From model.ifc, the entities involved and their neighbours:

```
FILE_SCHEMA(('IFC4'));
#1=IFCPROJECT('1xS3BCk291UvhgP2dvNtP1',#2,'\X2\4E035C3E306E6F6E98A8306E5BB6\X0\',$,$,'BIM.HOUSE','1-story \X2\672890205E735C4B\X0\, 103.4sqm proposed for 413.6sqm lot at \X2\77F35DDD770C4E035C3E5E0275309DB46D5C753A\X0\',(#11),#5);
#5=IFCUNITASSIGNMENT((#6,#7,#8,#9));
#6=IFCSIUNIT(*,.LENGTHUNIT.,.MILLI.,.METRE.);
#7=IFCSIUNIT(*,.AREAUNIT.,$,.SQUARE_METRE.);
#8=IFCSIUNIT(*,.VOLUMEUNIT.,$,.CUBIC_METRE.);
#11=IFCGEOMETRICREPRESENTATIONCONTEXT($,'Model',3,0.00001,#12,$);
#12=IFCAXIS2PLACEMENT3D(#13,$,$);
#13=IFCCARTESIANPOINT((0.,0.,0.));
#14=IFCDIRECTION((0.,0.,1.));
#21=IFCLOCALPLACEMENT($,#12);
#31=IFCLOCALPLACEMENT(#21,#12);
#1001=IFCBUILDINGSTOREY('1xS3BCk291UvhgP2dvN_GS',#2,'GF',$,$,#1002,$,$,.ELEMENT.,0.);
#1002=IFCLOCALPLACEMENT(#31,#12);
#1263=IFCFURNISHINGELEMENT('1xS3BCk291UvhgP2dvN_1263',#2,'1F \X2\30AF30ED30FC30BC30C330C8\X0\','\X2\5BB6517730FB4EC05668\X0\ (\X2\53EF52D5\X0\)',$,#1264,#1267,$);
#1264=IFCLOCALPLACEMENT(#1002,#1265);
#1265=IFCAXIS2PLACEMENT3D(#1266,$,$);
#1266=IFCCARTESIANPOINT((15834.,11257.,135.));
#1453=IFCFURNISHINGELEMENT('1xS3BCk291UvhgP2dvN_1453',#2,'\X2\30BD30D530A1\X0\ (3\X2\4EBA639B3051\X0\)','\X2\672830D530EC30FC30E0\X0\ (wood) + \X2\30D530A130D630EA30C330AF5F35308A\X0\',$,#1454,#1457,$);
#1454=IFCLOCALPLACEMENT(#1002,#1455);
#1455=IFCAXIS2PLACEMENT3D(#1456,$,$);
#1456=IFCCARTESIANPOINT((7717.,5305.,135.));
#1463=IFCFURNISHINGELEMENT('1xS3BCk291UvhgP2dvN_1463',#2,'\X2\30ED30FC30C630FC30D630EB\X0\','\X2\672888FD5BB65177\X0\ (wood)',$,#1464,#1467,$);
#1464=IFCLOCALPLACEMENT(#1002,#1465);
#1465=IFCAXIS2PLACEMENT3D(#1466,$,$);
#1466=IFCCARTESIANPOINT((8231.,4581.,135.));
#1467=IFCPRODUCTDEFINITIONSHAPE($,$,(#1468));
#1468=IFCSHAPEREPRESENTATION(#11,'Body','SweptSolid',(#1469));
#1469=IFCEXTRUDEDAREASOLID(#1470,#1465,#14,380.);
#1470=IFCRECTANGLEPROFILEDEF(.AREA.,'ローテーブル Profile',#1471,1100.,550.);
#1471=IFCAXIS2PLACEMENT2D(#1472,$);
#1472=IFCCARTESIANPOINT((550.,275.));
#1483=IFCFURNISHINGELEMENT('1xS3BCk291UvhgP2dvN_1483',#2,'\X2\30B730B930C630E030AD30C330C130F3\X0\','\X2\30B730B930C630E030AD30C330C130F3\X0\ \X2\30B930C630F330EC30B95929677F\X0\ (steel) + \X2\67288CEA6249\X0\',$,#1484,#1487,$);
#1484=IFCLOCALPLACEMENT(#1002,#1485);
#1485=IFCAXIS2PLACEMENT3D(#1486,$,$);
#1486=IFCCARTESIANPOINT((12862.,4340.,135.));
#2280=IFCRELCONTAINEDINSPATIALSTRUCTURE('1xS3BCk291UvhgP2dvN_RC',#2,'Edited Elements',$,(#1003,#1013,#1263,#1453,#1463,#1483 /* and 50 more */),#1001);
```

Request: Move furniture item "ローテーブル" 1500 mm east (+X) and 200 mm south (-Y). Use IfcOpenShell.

```python
import ifcopenshell
import ifcopenshell.api.geometry
import ifcopenshell.util.placement
import ifcopenshell.util.unit

model = ifcopenshell.open("model.ifc")
unit_scale = ifcopenshell.util.unit.calculate_unit_scale(model)

item = model.by_guid("1xS3BCk291UvhgP2dvN_1463")
matrix = ifcopenshell.util.placement.get_local_placement(item.ObjectPlacement)
matrix[0, 3] += 1.5 / unit_scale
matrix[1, 3] -= 0.2 / unit_scale
ifcopenshell.api.geometry.edit_object_placement(model, product=item, matrix=matrix, is_si=False)

print(ifcopenshell.util.placement.get_local_placement(item.ObjectPlacement).round(3) + 0.0)

model.write("model-out.ifc")
```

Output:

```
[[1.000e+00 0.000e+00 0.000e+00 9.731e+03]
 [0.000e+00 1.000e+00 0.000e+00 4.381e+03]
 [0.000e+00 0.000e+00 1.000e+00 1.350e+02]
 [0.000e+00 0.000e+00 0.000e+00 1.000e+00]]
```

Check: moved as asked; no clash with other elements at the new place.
